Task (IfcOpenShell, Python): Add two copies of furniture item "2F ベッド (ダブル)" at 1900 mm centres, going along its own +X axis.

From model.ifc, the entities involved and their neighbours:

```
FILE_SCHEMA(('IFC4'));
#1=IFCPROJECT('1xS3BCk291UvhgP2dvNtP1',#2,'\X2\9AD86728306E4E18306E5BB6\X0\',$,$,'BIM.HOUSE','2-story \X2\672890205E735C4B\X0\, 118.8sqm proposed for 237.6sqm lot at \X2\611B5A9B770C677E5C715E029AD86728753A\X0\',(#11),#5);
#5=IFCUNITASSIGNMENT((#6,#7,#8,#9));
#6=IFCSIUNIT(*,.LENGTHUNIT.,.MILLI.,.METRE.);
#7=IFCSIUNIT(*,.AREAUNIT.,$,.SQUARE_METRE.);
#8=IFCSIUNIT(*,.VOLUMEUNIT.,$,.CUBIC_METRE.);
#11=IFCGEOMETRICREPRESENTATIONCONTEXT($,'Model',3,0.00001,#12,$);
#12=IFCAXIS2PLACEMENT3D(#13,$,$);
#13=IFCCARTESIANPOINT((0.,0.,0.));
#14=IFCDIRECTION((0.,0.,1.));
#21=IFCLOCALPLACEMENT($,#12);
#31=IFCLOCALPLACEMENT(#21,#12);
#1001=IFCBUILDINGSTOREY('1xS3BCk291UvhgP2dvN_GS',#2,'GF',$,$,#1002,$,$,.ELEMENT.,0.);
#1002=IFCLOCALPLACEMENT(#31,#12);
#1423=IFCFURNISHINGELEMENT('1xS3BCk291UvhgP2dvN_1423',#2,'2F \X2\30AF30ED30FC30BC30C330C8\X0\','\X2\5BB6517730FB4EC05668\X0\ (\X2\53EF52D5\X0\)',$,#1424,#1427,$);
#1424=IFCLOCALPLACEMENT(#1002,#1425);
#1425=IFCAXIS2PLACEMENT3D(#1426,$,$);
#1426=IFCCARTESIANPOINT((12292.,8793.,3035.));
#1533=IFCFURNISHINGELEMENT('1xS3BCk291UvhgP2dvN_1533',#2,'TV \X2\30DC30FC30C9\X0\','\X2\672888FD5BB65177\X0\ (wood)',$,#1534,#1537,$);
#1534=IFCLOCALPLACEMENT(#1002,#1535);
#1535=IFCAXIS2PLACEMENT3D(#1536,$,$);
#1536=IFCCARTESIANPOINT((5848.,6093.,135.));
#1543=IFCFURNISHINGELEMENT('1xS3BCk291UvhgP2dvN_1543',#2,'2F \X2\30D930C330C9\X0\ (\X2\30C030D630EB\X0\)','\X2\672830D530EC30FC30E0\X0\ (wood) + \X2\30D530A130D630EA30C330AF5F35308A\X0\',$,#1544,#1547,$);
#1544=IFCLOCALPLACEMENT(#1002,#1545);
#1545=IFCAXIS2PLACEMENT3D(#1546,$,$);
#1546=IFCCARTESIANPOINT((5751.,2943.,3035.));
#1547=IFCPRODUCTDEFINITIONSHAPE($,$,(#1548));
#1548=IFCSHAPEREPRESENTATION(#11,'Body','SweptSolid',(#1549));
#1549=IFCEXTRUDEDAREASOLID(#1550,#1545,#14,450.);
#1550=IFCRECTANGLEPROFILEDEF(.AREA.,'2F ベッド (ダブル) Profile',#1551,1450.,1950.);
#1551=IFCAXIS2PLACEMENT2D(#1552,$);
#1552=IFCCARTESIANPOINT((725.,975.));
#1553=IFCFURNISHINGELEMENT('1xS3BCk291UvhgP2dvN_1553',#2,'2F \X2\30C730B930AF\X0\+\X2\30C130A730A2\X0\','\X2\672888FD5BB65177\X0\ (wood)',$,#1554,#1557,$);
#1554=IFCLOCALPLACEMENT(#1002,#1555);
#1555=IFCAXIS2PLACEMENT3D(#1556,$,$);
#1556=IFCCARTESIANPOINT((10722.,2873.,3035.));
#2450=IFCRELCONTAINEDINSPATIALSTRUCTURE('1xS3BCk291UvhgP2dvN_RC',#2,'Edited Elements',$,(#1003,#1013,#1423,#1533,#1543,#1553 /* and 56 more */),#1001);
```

```python
import ifcopenshell
import ifcopenshell.api.geometry
import ifcopenshell.api.root
import ifcopenshell.util.element
import ifcopenshell.util.placement
import ifcopenshell.util.unit

model = ifcopenshell.open("model.ifc")
unit_scale = ifcopenshell.util.unit.calculate_unit_scale(model)


def reuse_history(source, copy):
    """copy_class also copies each property set's owner history, people and application; keep the originals."""
    for rel in copy.IsDefinedBy:
        if rel.is_a("IfcRelDefinesByProperties") and (history := rel.RelatingPropertyDefinition.OwnerHistory):
            rel.RelatingPropertyDefinition.OwnerHistory = source.OwnerHistory
            ifcopenshell.util.element.remove_deep2(model, history)


source = model.by_id(1543)
base = ifcopenshell.util.placement.get_local_placement(source.ObjectPlacement)
step = base[:3, 0] * 1.9 / unit_scale

for i in range(1, 3):
    copy = ifcopenshell.api.root.copy_class(model, product=source)
    copy.Representation = ifcopenshell.util.element.copy_deep(
        model, source.Representation, exclude=["IfcGeometricRepresentationContext", "IfcRepresentationMap"]
    )
    reuse_history(source, copy)
    matrix = base.copy()
    matrix[:3, 3] += i * step
    print("added at", matrix[:3, 3].round(3) + 0.0)
    ifcopenshell.api.geometry.edit_object_placement(model, product=copy, matrix=matrix, is_si=False)

model.write("model_edited.ifc")
```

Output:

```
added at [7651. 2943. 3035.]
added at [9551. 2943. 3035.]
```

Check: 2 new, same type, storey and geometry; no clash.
